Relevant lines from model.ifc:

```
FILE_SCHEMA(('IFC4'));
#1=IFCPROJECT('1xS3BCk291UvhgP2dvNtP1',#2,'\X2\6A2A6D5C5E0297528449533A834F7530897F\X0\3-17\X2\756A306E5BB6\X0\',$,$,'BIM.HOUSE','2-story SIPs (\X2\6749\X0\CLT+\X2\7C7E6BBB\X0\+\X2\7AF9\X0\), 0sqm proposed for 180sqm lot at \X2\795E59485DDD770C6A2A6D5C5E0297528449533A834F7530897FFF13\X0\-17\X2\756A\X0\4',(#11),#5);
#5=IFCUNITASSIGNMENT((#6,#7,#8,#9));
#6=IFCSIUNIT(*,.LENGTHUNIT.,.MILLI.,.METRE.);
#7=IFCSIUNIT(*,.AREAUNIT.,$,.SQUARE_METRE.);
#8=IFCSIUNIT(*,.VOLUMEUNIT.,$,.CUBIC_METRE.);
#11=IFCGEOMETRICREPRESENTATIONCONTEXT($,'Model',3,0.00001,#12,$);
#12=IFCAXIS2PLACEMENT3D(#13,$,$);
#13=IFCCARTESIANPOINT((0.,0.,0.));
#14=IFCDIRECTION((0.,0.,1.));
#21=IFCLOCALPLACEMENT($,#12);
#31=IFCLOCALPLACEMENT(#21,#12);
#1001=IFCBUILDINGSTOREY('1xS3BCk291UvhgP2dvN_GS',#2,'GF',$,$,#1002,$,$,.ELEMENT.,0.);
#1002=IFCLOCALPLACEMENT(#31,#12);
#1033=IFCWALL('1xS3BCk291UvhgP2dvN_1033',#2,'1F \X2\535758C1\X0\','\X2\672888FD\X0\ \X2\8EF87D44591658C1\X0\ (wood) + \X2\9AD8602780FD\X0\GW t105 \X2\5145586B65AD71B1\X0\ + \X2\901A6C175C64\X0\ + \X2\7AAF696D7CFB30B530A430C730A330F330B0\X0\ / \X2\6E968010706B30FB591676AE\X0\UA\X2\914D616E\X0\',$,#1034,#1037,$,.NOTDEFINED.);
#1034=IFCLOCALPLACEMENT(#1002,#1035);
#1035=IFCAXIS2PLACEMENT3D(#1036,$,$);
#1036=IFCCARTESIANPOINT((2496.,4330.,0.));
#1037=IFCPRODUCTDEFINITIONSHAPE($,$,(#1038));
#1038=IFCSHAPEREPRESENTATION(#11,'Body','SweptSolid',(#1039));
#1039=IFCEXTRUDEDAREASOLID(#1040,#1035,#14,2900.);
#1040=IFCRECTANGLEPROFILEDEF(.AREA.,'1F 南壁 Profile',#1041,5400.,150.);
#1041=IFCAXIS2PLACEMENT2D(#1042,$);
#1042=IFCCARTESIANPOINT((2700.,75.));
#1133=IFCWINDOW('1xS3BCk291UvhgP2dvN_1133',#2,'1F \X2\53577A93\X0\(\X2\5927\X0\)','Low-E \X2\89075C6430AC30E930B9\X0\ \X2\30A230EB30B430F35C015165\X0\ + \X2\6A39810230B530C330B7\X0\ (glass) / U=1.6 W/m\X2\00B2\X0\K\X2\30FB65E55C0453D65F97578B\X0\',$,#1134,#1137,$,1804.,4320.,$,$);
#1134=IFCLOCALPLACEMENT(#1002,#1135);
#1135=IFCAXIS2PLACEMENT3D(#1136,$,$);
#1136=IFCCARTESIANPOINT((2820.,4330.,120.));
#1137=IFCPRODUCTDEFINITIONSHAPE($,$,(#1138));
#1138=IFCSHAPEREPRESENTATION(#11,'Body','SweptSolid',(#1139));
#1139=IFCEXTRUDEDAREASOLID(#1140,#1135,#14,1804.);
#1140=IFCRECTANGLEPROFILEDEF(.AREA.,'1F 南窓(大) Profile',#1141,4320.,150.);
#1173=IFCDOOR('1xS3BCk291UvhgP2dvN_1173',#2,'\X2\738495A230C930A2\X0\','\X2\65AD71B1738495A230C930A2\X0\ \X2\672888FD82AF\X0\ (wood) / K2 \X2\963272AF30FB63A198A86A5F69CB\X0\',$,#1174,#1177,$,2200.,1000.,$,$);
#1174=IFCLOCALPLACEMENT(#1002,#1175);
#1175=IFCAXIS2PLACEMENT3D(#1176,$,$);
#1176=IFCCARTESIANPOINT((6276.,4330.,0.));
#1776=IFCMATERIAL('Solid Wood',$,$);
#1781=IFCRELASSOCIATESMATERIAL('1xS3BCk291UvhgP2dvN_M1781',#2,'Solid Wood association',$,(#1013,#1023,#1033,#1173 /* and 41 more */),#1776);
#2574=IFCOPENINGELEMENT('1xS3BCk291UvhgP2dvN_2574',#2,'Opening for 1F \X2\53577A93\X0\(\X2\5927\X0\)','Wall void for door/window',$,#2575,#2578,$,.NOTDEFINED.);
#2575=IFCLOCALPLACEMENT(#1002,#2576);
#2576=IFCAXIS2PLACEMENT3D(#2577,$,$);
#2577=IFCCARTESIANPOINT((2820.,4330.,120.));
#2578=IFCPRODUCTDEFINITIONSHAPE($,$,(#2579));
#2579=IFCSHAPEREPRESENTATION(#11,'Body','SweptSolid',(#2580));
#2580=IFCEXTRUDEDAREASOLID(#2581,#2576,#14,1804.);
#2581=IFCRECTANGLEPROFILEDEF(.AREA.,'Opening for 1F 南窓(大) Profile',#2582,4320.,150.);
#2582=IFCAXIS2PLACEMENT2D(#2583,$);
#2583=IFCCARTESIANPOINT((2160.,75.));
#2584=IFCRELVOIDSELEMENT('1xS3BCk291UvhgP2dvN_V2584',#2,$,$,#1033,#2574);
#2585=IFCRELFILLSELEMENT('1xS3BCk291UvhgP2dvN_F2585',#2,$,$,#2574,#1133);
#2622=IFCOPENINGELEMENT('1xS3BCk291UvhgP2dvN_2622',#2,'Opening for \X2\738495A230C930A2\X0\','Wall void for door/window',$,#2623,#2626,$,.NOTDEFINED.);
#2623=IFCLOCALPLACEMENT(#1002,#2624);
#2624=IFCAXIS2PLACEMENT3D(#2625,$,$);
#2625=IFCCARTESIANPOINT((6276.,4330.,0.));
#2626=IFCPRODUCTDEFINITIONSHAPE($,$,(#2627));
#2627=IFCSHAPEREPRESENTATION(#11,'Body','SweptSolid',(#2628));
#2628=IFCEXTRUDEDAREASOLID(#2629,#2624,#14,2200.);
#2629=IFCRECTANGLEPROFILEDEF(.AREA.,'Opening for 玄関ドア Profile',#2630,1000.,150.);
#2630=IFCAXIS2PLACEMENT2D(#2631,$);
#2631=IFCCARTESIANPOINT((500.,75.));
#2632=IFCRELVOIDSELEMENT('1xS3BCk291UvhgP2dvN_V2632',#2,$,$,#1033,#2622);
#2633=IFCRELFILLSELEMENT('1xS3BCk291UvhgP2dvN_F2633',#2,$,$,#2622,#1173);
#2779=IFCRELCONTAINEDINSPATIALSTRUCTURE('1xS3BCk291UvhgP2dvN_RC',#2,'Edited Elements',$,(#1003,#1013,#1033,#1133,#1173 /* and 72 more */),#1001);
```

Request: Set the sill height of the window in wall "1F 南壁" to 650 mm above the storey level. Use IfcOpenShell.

```python
import numpy as np
import ifcopenshell
import ifcopenshell.api.geometry
import ifcopenshell.geom
import ifcopenshell.util.element
import ifcopenshell.util.placement
import ifcopenshell.util.shape
import ifcopenshell.util.unit

model = ifcopenshell.open("model.ifc")
unit_scale = ifcopenshell.util.unit.calculate_unit_scale(model)

window = model.by_guid("1xS3BCk291UvhgP2dvN_1133")
opening = window.FillsVoids[0].RelatingOpeningElement
storey = ifcopenshell.util.element.get_container(window, ifc_class="IfcBuildingStorey")
level = ifcopenshell.util.placement.get_local_placement(storey.ObjectPlacement)[2, 3]

# The opening's origin need not be at the sill, so measure its lowest point.
shape = ifcopenshell.geom.create_shape(ifcopenshell.geom.settings(), opening)
bottom = ifcopenshell.util.shape.get_shape_bottom_elevation(shape, shape.geometry) / unit_scale
dz = level + 650.0 - bottom

shift = np.array([0.0, 0.0, dz])
# The window is not placed relative to its opening, so move both.
for product in (opening, window):
    matrix = ifcopenshell.util.placement.get_local_placement(product.ObjectPlacement)
    matrix[:3, 3] += shift
    ifcopenshell.api.geometry.edit_object_placement(model, product=product, matrix=matrix, is_si=False)

print(f"moved by {dz * unit_scale:+.3f} m")

model.write("model-out.ifc")
```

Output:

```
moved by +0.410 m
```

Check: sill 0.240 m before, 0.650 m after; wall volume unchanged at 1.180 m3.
